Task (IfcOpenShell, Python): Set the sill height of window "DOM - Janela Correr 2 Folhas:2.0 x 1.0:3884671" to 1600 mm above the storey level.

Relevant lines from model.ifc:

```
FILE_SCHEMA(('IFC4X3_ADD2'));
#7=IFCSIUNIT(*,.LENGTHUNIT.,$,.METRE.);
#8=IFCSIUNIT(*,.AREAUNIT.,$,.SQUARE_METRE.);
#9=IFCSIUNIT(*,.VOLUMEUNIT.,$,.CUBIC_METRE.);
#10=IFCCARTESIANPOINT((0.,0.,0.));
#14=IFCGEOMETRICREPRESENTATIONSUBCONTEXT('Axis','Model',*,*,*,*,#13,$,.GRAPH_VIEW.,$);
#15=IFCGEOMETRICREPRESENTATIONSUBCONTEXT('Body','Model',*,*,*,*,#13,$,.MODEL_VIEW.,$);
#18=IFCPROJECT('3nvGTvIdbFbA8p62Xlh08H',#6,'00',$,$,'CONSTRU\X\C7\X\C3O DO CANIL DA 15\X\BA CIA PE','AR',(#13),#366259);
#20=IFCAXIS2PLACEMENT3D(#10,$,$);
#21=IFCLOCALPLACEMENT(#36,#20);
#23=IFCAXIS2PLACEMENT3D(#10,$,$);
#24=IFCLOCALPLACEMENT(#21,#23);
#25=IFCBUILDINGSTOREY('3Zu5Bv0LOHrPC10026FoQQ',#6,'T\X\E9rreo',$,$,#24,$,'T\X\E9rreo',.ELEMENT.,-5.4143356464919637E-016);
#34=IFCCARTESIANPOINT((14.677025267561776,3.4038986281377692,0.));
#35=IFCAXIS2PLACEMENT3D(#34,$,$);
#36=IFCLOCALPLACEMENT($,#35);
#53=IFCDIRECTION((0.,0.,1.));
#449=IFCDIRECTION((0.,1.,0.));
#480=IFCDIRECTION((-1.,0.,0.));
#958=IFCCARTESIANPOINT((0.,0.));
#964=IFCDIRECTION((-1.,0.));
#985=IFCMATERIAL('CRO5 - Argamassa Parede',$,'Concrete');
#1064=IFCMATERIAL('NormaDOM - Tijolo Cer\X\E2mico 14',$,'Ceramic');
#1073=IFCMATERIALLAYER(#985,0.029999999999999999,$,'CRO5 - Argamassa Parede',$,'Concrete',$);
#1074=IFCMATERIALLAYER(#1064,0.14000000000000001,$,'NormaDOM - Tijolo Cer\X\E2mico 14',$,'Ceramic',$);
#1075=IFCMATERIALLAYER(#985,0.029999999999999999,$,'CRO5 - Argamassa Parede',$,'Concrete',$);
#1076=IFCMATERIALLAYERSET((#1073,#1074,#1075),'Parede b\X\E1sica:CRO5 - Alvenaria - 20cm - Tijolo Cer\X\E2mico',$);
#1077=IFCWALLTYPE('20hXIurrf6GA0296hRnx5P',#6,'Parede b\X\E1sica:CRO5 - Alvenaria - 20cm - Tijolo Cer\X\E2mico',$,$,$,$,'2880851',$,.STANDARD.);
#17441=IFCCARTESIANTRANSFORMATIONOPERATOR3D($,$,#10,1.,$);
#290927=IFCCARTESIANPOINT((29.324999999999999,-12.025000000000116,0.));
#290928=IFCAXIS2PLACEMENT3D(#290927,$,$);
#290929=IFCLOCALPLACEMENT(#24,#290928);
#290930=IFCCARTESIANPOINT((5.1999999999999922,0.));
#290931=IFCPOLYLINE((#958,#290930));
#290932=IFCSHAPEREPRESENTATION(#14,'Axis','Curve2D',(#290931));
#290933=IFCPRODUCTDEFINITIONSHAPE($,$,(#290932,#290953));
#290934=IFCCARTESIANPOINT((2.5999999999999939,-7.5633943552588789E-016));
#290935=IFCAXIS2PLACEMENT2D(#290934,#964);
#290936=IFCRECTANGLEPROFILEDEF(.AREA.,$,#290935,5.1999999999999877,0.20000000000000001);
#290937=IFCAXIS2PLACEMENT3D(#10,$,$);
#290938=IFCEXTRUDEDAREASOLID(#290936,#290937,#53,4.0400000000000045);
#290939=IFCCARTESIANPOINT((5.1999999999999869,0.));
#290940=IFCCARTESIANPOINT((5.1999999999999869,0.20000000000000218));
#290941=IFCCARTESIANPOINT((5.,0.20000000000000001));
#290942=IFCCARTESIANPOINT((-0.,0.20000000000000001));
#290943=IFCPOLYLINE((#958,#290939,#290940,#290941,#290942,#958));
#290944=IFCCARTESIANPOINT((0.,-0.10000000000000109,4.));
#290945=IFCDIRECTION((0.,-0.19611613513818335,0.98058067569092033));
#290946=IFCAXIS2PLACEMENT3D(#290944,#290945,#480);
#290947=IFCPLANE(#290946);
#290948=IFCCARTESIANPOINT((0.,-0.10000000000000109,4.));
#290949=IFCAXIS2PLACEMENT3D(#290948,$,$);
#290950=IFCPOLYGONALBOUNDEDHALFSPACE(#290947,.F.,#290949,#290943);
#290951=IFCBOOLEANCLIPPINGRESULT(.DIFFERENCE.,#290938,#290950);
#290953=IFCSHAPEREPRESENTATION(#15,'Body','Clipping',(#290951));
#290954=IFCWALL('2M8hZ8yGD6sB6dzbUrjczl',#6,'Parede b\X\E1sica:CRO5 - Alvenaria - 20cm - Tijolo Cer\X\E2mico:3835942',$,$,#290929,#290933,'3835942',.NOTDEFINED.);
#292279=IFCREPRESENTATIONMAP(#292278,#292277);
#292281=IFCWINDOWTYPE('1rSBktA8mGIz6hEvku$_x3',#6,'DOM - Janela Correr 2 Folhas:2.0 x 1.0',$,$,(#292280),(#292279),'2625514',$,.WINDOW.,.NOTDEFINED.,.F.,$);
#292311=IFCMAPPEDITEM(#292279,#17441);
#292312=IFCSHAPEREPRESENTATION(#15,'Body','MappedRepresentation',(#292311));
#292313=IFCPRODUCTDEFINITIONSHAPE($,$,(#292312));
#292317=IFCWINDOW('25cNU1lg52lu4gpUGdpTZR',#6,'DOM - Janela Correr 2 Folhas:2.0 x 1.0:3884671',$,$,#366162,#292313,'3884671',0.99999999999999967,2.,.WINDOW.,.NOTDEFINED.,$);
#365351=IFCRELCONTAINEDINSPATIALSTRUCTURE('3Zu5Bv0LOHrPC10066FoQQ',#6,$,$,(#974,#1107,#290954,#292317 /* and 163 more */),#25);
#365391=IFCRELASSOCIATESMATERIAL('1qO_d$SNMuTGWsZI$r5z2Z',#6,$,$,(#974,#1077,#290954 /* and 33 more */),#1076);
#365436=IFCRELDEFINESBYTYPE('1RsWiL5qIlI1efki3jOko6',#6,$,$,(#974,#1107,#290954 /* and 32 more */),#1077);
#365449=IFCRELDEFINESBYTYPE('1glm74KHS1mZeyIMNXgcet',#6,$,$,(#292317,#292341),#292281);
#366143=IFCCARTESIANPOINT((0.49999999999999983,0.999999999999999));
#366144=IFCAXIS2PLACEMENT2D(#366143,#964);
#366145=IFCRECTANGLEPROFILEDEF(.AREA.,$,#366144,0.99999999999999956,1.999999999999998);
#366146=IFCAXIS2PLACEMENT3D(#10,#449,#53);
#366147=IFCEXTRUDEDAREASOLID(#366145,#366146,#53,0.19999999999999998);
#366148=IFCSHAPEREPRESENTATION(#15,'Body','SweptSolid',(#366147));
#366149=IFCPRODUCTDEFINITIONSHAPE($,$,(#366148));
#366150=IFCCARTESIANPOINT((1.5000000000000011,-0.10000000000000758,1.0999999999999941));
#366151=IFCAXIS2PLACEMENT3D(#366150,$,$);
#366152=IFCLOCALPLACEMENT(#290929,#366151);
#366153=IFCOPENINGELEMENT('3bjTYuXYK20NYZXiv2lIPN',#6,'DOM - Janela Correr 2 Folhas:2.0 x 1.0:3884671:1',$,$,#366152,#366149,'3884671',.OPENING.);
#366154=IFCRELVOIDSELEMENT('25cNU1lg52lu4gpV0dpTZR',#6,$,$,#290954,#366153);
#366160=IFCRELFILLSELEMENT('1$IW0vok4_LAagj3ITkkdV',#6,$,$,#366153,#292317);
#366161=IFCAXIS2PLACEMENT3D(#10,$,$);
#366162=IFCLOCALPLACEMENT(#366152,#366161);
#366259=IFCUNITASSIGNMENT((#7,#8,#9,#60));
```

```python
import numpy as np
import ifcopenshell
import ifcopenshell.api.geometry
import ifcopenshell.geom
import ifcopenshell.util.element
import ifcopenshell.util.placement
import ifcopenshell.util.shape
import ifcopenshell.util.unit

model = ifcopenshell.open("model.ifc")
unit_scale = ifcopenshell.util.unit.calculate_unit_scale(model)

window = model.by_guid("25cNU1lg52lu4gpUGdpTZR")
opening = window.FillsVoids[0].RelatingOpeningElement
storey = ifcopenshell.util.element.get_container(window, ifc_class="IfcBuildingStorey")
level = ifcopenshell.util.placement.get_local_placement(storey.ObjectPlacement)[2, 3]

# The opening's origin need not be at the sill, so measure its lowest point.
shape = ifcopenshell.geom.create_shape(ifcopenshell.geom.settings(), opening)
bottom = ifcopenshell.util.shape.get_shape_bottom_elevation(shape, shape.geometry) / unit_scale
dz = level + 1.6 - bottom

shift = np.array([0.0, 0.0, dz])
# The window is placed relative to its opening, so it follows when the opening moves.
matrix = ifcopenshell.util.placement.get_local_placement(opening.ObjectPlacement)
matrix[:3, 3] += shift
ifcopenshell.api.geometry.edit_object_placement(
    model, product=opening, matrix=matrix, is_si=False, should_transform_children=True
)

print(f"moved by {dz * unit_scale:+.3f} m")

model.write("model-out.ifc")
```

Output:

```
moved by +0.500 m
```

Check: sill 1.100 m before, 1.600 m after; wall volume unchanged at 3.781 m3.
